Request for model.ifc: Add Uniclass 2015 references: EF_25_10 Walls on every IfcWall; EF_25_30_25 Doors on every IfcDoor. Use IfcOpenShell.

First a look at what the model holds.

```python
import ifcopenshell

model = ifcopenshell.open("model.ifc")
print(model.schema)
print("classifications:", [c.Name for c in model.by_type("IfcClassification")])
for ifc_class in ("IfcDoor", "IfcRoof", "IfcStair", "IfcWall", "IfcWindow"):
    print(ifc_class, len(model.by_type(ifc_class)))
```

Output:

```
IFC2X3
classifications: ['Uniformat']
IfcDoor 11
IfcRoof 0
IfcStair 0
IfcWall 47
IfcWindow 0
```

```python
import ifcopenshell
import ifcopenshell.api.classification

model = ifcopenshell.open("model.ifc")

# IFC2X3 requires Source and Edition and has no link from the project to the system.
system = model.create_entity("IfcClassification", Source="NBS", Edition="2015", Name="Uniclass 2015")

codes = {
    "IfcWall": ("EF_25_10", "Walls"),
    "IfcDoor": ("EF_25_30_25", "Doors"),
}
for ifc_class, (code, name) in codes.items():
    products = model.by_type(ifc_class)
    ifcopenshell.api.classification.add_reference(
        model, products=products, classification=system, identification=code, name=name
    )
    print(code, len(products))

model.write("model_v2.ifc")
```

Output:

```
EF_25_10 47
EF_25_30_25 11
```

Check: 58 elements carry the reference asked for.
